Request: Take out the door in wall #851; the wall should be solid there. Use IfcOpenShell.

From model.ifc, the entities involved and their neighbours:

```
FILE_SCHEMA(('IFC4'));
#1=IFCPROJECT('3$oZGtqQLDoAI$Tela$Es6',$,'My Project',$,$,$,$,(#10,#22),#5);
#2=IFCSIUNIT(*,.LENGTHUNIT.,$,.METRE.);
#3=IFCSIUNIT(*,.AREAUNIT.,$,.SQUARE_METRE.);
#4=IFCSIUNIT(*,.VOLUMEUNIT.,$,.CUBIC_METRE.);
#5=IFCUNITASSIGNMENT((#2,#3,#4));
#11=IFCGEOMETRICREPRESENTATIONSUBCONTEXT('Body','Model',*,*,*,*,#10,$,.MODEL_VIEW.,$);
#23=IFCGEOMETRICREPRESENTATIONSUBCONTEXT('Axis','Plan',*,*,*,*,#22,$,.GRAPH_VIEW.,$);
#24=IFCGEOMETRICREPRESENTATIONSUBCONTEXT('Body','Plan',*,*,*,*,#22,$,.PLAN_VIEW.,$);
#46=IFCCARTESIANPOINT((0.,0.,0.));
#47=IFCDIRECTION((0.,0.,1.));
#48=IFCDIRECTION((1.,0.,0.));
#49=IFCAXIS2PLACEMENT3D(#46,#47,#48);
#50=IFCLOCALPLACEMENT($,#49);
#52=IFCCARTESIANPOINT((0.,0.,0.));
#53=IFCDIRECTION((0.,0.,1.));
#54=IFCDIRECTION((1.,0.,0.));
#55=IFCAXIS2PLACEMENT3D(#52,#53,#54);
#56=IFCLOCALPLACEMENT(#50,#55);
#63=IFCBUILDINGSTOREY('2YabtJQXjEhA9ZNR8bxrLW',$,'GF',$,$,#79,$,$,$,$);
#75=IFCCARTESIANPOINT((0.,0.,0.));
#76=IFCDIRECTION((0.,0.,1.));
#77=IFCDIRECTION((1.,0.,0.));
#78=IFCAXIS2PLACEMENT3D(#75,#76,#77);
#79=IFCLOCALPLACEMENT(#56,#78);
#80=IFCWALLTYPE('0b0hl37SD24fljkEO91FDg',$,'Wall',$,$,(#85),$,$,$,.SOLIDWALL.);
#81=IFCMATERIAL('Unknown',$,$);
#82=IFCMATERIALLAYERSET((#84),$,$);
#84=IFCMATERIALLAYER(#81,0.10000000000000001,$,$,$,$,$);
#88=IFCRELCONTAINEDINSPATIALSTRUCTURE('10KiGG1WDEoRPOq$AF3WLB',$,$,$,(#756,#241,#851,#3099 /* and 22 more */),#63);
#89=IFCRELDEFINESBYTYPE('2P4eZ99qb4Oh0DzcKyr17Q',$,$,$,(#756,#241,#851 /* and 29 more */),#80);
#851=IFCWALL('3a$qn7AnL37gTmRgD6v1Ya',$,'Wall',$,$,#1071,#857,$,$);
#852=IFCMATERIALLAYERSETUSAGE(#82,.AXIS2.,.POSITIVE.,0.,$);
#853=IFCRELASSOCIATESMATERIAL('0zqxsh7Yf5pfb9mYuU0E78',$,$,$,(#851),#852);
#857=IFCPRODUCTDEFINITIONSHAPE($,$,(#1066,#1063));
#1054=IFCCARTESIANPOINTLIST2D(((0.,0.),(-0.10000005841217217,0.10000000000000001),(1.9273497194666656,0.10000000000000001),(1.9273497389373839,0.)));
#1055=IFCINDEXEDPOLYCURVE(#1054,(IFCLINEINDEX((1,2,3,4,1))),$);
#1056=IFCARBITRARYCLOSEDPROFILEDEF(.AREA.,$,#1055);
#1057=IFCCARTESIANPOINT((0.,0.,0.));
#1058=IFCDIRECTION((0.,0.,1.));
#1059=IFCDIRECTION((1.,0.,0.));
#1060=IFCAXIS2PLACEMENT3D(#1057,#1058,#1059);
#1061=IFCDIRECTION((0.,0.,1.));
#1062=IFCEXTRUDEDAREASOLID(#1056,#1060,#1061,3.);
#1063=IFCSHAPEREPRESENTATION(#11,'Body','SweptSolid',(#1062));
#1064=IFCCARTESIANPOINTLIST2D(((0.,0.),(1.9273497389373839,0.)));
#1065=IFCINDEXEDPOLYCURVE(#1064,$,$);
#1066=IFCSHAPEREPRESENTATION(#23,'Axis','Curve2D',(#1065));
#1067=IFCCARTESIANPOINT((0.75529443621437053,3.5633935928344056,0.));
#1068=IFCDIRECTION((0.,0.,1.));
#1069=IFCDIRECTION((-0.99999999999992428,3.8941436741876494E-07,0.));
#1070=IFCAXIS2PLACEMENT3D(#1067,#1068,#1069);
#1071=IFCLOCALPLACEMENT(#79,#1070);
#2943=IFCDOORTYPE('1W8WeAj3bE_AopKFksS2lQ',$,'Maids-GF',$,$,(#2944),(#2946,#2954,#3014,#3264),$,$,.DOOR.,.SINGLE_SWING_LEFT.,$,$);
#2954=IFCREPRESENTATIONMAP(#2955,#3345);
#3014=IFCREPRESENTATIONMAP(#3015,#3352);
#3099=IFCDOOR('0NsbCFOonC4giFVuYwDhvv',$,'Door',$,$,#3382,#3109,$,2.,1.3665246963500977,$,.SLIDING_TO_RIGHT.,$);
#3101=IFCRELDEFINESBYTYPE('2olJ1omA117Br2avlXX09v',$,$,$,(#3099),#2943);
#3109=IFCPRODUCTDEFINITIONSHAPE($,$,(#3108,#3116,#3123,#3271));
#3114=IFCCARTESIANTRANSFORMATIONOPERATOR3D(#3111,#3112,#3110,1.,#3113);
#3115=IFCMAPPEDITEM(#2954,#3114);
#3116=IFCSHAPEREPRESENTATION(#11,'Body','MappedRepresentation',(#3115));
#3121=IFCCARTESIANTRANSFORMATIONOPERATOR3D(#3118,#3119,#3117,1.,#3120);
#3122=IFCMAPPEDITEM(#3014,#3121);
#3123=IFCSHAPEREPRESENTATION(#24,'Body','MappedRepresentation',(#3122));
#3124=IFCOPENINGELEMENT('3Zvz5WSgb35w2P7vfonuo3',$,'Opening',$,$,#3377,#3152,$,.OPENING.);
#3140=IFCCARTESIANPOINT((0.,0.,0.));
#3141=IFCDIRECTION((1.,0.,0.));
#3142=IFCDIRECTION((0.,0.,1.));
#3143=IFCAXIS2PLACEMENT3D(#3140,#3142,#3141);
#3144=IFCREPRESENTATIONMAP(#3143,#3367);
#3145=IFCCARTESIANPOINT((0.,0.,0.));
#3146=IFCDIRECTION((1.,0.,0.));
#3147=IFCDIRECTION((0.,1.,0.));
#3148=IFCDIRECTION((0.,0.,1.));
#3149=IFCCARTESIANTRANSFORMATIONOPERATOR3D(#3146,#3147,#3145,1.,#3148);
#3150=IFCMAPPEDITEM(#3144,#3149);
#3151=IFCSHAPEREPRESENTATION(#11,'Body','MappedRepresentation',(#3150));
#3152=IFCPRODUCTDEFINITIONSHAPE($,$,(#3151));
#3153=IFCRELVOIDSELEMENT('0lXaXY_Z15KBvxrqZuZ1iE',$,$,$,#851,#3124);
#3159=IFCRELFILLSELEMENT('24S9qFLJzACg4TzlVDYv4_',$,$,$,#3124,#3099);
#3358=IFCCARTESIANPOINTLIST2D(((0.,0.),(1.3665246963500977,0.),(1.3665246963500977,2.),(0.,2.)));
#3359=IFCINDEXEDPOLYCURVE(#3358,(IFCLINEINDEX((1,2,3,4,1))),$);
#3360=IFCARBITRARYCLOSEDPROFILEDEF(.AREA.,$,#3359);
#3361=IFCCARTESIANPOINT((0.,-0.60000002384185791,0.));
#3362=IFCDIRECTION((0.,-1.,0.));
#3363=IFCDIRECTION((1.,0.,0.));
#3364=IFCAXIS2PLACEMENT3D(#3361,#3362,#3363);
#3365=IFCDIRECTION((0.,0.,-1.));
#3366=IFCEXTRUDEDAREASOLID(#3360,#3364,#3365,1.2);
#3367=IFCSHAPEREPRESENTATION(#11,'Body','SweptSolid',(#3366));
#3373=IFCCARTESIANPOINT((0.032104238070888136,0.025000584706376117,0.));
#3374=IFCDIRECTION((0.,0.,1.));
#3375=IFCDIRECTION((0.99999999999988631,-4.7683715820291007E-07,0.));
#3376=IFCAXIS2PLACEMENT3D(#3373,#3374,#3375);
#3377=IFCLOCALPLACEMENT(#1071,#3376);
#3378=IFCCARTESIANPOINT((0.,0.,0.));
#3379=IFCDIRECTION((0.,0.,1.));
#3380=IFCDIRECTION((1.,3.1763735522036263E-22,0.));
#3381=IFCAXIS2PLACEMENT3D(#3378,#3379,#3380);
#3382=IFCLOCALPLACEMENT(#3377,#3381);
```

```python
import ifcopenshell
import ifcopenshell.api.feature
import ifcopenshell.api.root
import ifcopenshell.geom
import ifcopenshell.util.shape

model = ifcopenshell.open("model.ifc")
settings = ifcopenshell.geom.settings()


def volume(element):
    """Net volume in cubic metres, openings subtracted."""
    shape = ifcopenshell.geom.create_shape(settings, element)
    return ifcopenshell.util.shape.get_volume(shape.geometry)


door = model.by_guid("0NsbCFOonC4giFVuYwDhvv")
opening = door.FillsVoids[0].RelatingOpeningElement
wall = opening.VoidsElements[0].RelatingBuildingElement
before = volume(wall)

ifcopenshell.api.root.remove_product(model, product=door)
ifcopenshell.api.feature.remove_feature(model, feature=opening)

after = volume(wall)

print(f"wall volume {before:.3f} -> {after:.3f} m3")

model.write("model_edited.ifc")
```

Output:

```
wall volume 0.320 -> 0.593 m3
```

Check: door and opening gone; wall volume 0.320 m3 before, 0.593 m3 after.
